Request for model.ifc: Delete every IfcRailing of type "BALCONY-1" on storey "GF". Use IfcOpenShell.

First a look at what the model holds.

```python
import ifcopenshell
import ifcopenshell.util.element

model = ifcopenshell.open("model.ifc")
print(model.schema)
storey = next(s for s in model.by_type("IfcBuildingStorey") if s.Name == "GF")
railings = [e for e in ifcopenshell.util.element.get_decomposition(storey) if e.is_a("IfcRailing")]
seen = {}
for e in railings:
    element_type = ifcopenshell.util.element.get_type(e)
    name = element_type.Name if element_type not in (None, e) else None
    seen[name] = seen.get(name, 0) + 1
for name, count in sorted(seen.items(), key=str):
    print(count, "x", name)
```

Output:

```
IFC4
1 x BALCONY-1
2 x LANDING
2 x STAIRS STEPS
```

```python
import ifcopenshell
import ifcopenshell.api.root
import ifcopenshell.util.element

model = ifcopenshell.open("model.ifc")

storey = next(s for s in model.by_type("IfcBuildingStorey") if s.Name == "GF")
railings = [e for e in ifcopenshell.util.element.get_decomposition(storey) if e.is_a("IfcRailing")]
targets = [e for e in railings if (t := ifcopenshell.util.element.get_type(e)) not in (None, e) and t.Name == "BALCONY-1"]

for e in targets:
    ifcopenshell.api.root.remove_product(model, product=e)
print(len(targets), "removed")

model.write("model_rev.ifc")
```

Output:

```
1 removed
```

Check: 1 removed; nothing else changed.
